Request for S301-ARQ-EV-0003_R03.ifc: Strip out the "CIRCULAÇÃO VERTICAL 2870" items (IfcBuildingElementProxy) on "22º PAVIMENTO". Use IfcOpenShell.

First a look at what the model holds.

```python
import ifcopenshell
import ifcopenshell.util.element

model = ifcopenshell.open("S301-ARQ-EV-0003_R03.ifc")
print(model.schema)
storey = next(s for s in model.by_type("IfcBuildingStorey") if s.Name == "22º PAVIMENTO")
proxies = [e for e in ifcopenshell.util.element.get_decomposition(storey) if e.is_a("IfcBuildingElementProxy")]
seen = {}
for e in proxies:
    element_type = ifcopenshell.util.element.get_type(e)
    name = element_type.Name if element_type not in (None, e) else None
    seen[name] = seen.get(name, 0) + 1
for name, count in sorted(seen.items(), key=str):
    print(count, "x", name)
```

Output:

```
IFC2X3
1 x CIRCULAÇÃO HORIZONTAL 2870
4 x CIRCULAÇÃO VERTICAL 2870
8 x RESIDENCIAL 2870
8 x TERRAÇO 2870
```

```python
import ifcopenshell
import ifcopenshell.api.root
import ifcopenshell.util.element

model = ifcopenshell.open("S301-ARQ-EV-0003_R03.ifc")

storey = next(s for s in model.by_type("IfcBuildingStorey") if s.Name == "22º PAVIMENTO")
proxies = [e for e in ifcopenshell.util.element.get_decomposition(storey) if e.is_a("IfcBuildingElementProxy")]
targets = [e for e in proxies if (t := ifcopenshell.util.element.get_type(e)) not in (None, e) and t.Name == "CIRCULAÇÃO VERTICAL 2870"]

for e in targets:
    ifcopenshell.api.root.remove_product(model, product=e)
print(len(targets), "removed")

model.write("S301-ARQ-EV-0003_R03_updated.ifc")
```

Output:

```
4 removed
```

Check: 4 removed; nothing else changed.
